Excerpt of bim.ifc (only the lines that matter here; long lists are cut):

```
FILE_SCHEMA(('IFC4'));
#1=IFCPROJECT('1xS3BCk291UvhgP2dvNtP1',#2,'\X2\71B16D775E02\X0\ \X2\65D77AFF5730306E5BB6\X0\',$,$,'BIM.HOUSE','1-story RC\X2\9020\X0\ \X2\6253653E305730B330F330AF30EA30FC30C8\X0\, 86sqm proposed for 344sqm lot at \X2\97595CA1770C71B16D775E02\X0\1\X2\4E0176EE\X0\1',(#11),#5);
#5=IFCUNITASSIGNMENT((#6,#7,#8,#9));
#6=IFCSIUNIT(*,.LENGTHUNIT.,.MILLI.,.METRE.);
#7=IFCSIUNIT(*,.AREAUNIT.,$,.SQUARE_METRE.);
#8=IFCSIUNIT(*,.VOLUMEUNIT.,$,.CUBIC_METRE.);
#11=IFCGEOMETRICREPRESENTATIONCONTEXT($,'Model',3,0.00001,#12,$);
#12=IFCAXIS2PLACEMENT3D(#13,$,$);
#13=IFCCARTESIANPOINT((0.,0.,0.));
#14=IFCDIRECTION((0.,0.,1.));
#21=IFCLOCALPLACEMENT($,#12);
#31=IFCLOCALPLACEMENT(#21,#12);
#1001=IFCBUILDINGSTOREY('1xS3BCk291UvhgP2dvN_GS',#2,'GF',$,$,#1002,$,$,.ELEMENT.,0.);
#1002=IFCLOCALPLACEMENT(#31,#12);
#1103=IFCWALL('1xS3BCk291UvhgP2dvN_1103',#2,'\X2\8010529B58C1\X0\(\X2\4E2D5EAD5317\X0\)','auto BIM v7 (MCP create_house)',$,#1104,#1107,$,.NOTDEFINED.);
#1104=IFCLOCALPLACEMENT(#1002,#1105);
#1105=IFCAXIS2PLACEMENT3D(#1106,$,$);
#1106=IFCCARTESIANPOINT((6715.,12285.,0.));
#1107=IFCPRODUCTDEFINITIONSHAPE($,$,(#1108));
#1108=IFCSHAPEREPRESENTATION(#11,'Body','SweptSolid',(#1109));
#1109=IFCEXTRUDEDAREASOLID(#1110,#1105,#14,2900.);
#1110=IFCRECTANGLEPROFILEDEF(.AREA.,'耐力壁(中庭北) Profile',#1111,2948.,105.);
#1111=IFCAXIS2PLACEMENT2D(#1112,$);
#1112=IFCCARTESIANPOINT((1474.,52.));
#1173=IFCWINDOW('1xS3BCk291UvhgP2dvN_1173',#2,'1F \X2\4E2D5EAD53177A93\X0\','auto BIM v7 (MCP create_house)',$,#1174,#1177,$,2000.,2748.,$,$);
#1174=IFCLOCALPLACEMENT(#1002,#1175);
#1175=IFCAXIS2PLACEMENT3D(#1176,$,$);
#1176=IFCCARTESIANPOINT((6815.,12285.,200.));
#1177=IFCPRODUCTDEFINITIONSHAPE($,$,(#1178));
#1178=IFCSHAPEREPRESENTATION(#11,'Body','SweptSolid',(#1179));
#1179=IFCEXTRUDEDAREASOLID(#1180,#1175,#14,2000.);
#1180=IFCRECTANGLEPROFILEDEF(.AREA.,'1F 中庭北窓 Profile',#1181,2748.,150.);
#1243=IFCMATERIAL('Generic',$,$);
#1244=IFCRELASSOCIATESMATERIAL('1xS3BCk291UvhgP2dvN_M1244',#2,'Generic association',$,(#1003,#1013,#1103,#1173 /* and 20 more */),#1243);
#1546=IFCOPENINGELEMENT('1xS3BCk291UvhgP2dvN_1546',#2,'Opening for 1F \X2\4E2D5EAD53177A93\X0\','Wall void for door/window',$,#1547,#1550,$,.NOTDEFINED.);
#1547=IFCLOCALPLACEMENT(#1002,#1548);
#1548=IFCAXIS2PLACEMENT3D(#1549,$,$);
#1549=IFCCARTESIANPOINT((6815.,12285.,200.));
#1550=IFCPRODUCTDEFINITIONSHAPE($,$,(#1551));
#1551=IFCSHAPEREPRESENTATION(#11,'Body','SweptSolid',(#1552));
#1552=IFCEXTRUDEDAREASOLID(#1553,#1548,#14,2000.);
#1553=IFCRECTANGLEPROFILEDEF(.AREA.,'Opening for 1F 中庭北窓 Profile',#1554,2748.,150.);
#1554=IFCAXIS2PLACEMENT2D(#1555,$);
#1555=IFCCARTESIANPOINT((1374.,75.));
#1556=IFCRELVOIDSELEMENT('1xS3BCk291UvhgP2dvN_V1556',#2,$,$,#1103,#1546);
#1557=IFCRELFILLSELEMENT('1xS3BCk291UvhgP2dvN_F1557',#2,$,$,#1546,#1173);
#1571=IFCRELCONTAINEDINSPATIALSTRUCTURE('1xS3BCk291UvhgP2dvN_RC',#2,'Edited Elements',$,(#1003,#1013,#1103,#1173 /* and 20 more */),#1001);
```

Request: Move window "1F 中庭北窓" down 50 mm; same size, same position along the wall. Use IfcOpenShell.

```python
import numpy as np
import ifcopenshell
import ifcopenshell.api.geometry
import ifcopenshell.util.placement
import ifcopenshell.util.unit

model = ifcopenshell.open("bim.ifc")
unit_scale = ifcopenshell.util.unit.calculate_unit_scale(model)

window = model.by_guid("1xS3BCk291UvhgP2dvN_1173")
opening = window.FillsVoids[0].RelatingOpeningElement
dz = -0.05 / unit_scale

shift = np.array([0.0, 0.0, dz])
# The window is not placed relative to its opening, so move both.
for product in (opening, window):
    matrix = ifcopenshell.util.placement.get_local_placement(product.ObjectPlacement)
    matrix[:3, 3] += shift
    ifcopenshell.api.geometry.edit_object_placement(model, product=product, matrix=matrix, is_si=False)

print(f"moved by {dz * unit_scale:+.3f} m")

model.write("bim_updated.ifc")
```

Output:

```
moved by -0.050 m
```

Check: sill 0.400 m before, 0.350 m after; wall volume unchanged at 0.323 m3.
